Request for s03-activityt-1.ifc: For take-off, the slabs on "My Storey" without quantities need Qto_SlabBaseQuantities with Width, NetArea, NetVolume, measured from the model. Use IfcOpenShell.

First a look at what the model holds.

```python
import ifcopenshell
import ifcopenshell.util.element
import ifcopenshell.util.unit

model = ifcopenshell.open("s03-activityt-1.ifc")
print(model.schema)
for unit_type in ("LENGTHUNIT", "AREAUNIT", "VOLUMEUNIT"):
    print(unit_type, ifcopenshell.util.unit.calculate_unit_scale(model, unit_type))
storey = next(s for s in model.by_type("IfcBuildingStorey") if s.Name == "My Storey")
slabs = [e for e in ifcopenshell.util.element.get_decomposition(storey) if e.is_a("IfcSlab")]
for e in sorted(slabs, key=lambda e: e.id()):
    print(e.id(), e.is_a(), e.Name, list(ifcopenshell.util.element.get_psets(e, qtos_only=True)), sep=" | ")
```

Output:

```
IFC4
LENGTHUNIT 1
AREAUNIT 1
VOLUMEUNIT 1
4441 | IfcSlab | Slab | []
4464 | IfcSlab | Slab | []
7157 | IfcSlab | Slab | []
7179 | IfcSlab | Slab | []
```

```python
import ifcopenshell
import ifcopenshell.api.pset
import ifcopenshell.geom
import ifcopenshell.util.element
import ifcopenshell.util.shape
import ifcopenshell.util.unit

model = ifcopenshell.open("s03-activityt-1.ifc")
unit_scale = ifcopenshell.util.unit.calculate_unit_scale(model)
area_scale = ifcopenshell.util.unit.calculate_unit_scale(model, "AREAUNIT")
volume_scale = ifcopenshell.util.unit.calculate_unit_scale(model, "VOLUMEUNIT")
settings = ifcopenshell.geom.settings()

storey = next(s for s in model.by_type("IfcBuildingStorey") if s.Name == "My Storey")
slabs = [e for e in ifcopenshell.util.element.get_decomposition(storey) if e.is_a("IfcSlab")]

for e in sorted(slabs, key=lambda e: e.id()):
    if ifcopenshell.util.element.get_psets(e, qtos_only=True, should_inherit=False):
        continue
    # Geometry comes back in metres, in the element's own axes.
    shape = ifcopenshell.geom.create_shape(settings, e)
    values = {
        "Width": ifcopenshell.util.shape.get_z(shape.geometry) / unit_scale,
        "NetArea": ifcopenshell.util.shape.get_footprint_area(shape.geometry) / area_scale,
        "NetVolume": ifcopenshell.util.shape.get_volume(shape.geometry) / volume_scale,
    }
    qto = ifcopenshell.api.pset.add_qto(model, product=e, name="Qto_SlabBaseQuantities")
    ifcopenshell.api.pset.edit_qto(model, qto=qto, properties=values)
    print(e.id(), {k: round(v, 3) for k, v in values.items()})

model.write("s03-activityt-1-out.ifc")
```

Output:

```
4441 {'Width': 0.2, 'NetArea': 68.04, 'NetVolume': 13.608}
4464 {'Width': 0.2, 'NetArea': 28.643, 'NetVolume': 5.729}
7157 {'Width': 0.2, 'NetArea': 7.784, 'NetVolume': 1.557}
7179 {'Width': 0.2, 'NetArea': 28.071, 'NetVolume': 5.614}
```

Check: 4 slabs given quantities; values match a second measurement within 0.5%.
